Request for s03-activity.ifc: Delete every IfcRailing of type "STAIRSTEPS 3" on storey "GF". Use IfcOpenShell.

First a look at what the model holds.

```python
import ifcopenshell
import ifcopenshell.util.element

model = ifcopenshell.open("s03-activity.ifc")
print(model.schema)
storey = next(s for s in model.by_type("IfcBuildingStorey") if s.Name == "GF")
railings = [e for e in ifcopenshell.util.element.get_decomposition(storey) if e.is_a("IfcRailing")]
seen = {}
for e in railings:
    element_type = ifcopenshell.util.element.get_type(e)
    name = element_type.Name if element_type not in (None, e) else None
    seen[name] = seen.get(name, 0) + 1
for name, count in sorted(seen.items(), key=str):
    print(count, "x", name)
```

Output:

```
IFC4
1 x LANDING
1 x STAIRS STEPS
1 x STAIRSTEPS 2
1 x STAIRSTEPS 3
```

```python
import ifcopenshell
import ifcopenshell.api.root
import ifcopenshell.util.element

model = ifcopenshell.open("s03-activity.ifc")

storey = next(s for s in model.by_type("IfcBuildingStorey") if s.Name == "GF")
railings = [e for e in ifcopenshell.util.element.get_decomposition(storey) if e.is_a("IfcRailing")]
targets = [e for e in railings if (t := ifcopenshell.util.element.get_type(e)) not in (None, e) and t.Name == "STAIRSTEPS 3"]

for e in targets:
    ifcopenshell.api.root.remove_product(model, product=e)
print(len(targets), "removed")

model.write("s03-activity_updated.ifc")
```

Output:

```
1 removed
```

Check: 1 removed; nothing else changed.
